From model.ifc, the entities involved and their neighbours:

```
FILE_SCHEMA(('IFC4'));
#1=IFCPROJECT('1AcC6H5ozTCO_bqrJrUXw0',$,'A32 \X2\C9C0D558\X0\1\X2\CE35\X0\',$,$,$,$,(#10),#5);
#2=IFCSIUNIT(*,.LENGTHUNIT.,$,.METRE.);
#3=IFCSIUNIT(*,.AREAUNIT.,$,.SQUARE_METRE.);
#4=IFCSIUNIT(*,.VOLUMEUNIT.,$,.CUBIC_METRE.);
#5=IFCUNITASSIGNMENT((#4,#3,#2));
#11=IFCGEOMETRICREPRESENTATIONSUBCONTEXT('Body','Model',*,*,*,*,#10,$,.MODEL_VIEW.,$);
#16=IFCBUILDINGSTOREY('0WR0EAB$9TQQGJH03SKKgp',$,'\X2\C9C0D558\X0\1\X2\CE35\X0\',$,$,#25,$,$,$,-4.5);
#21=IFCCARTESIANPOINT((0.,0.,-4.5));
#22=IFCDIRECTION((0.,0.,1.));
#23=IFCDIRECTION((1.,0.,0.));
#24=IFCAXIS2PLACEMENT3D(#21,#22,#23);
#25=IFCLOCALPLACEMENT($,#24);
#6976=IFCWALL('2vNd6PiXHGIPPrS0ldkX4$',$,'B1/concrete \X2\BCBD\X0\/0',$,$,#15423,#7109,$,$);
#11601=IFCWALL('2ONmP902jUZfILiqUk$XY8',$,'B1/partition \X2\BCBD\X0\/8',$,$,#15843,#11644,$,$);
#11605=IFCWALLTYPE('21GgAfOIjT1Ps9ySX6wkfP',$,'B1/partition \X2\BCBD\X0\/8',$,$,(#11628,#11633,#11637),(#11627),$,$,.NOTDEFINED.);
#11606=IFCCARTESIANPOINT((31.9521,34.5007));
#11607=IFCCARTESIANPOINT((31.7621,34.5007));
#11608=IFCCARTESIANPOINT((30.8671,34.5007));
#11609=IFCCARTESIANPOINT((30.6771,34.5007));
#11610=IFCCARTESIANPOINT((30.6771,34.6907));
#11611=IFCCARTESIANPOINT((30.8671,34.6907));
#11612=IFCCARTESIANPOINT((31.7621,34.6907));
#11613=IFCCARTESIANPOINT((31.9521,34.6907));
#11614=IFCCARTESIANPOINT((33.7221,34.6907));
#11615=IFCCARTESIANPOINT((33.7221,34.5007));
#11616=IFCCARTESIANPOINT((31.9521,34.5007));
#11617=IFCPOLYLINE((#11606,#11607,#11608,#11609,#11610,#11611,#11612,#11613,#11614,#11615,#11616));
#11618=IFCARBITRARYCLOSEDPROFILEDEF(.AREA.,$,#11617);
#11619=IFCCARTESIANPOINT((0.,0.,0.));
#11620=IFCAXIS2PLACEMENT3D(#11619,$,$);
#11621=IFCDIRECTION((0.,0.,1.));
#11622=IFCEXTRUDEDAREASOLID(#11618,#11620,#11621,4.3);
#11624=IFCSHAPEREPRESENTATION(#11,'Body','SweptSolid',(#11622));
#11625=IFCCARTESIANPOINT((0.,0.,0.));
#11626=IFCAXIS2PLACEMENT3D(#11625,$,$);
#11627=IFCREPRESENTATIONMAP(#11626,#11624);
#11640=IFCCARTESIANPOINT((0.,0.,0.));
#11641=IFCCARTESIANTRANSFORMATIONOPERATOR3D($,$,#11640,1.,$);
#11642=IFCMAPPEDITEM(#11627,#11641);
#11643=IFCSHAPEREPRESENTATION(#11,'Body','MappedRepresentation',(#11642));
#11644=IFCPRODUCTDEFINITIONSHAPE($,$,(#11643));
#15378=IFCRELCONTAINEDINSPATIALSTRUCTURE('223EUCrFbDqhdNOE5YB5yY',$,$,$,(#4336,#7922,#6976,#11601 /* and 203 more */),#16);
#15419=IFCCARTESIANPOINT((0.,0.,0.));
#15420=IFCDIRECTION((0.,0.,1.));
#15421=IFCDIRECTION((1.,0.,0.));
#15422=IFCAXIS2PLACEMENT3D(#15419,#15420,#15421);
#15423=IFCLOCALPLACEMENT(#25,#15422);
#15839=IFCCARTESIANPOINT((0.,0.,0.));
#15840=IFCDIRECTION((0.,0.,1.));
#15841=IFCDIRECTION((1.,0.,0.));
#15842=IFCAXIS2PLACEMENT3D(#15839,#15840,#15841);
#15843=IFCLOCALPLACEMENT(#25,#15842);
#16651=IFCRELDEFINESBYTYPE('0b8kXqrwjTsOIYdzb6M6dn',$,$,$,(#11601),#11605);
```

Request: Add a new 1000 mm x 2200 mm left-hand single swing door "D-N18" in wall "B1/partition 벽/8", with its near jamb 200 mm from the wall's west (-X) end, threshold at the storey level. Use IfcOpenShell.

```python
import numpy as np
import ifcopenshell
import ifcopenshell.api.feature
import ifcopenshell.api.geometry
import ifcopenshell.api.root
import ifcopenshell.api.spatial
import ifcopenshell.geom
import ifcopenshell.util.element
import ifcopenshell.util.placement
import ifcopenshell.util.representation
import ifcopenshell.util.shape
import ifcopenshell.util.unit

model = ifcopenshell.open("model.ifc")
unit_scale = ifcopenshell.util.unit.calculate_unit_scale(model)
settings = ifcopenshell.geom.settings()


def volume(element):
    """Net volume in cubic metres, openings subtracted."""
    shape = ifcopenshell.geom.create_shape(settings, element)
    return ifcopenshell.util.shape.get_volume(shape.geometry)


wall = model.by_id(11601)
storey = ifcopenshell.util.element.get_container(wall, ifc_class="IfcBuildingStorey")
context = ifcopenshell.util.representation.get_context(model, "Model", "Body", "MODEL_VIEW")
before = volume(wall)

width, height, from_end, sill = 1, 2.2, 0.2, 0.0  # metres

# The wall runs along its own X axis, and the end named is its -X end.
wall_shape = ifcopenshell.geom.create_shape(settings, wall)
x, y, z = ifcopenshell.util.shape.get_vertices(wall_shape.geometry).T
start = x.min() + from_end
face, thickness = float(y.min()), float(y.max() - y.min())
wall_matrix = ifcopenshell.util.placement.get_local_placement(wall.ObjectPlacement)
level = ifcopenshell.util.placement.get_local_placement(storey.ObjectPlacement)[2, 3]


def in_wall(x, y):
    """Placement at x, y metres in the wall's axes, at sill height."""
    matrix = wall_matrix.copy()
    matrix[:, 3] = wall_matrix @ np.array([x / unit_scale, y / unit_scale, 0.0, 1.0])
    matrix[2, 3] = level + sill / unit_scale
    return matrix


# Opening: a box that overshoots both wall faces by 50 mm.
opening = ifcopenshell.api.root.create_entity(model, ifc_class="IfcOpeningElement", predefined_type="OPENING")
box = ifcopenshell.api.geometry.add_wall_representation(
    model, context=context, length=width, height=height, thickness=thickness + 0.1
)
ifcopenshell.api.geometry.assign_representation(model, product=opening, representation=box)
ifcopenshell.api.geometry.edit_object_placement(model, product=opening, matrix=in_wall(start, face - 0.05), is_si=False)
ifcopenshell.api.feature.add_feature(model, feature=opening, element=wall)

door = ifcopenshell.api.root.create_entity(model, ifc_class="IfcDoor", name="D-N18", predefined_type="DOOR")
door.OverallWidth, door.OverallHeight = width / unit_scale, height / unit_scale
door.OperationType = "SINGLE_SWING_LEFT"
body = ifcopenshell.api.geometry.add_door_representation(
    model,
    context=context,
    overall_width=door.OverallWidth,
    overall_height=door.OverallHeight,
    operation_type="SINGLE_SWING_LEFT",
    lining_properties={"LiningDepth": thickness / unit_scale, "ThresholdDepth": thickness / unit_scale},
)
ifcopenshell.api.geometry.assign_representation(model, product=door, representation=body)
ifcopenshell.api.spatial.assign_container(model, products=[door], relating_structure=storey)
ifcopenshell.api.feature.add_filling(model, opening=opening, element=door)

# The lining spans the wall, so the door starts at the wall face.
ifcopenshell.api.geometry.edit_object_placement(model, product=door, matrix=in_wall(start, face), is_si=False)

after = volume(wall)

print(f"wall volume {before:.3f} -> {after:.3f} m3")

model.write("model-out.ifc")
```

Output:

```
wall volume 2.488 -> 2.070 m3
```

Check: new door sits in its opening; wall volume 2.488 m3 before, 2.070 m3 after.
